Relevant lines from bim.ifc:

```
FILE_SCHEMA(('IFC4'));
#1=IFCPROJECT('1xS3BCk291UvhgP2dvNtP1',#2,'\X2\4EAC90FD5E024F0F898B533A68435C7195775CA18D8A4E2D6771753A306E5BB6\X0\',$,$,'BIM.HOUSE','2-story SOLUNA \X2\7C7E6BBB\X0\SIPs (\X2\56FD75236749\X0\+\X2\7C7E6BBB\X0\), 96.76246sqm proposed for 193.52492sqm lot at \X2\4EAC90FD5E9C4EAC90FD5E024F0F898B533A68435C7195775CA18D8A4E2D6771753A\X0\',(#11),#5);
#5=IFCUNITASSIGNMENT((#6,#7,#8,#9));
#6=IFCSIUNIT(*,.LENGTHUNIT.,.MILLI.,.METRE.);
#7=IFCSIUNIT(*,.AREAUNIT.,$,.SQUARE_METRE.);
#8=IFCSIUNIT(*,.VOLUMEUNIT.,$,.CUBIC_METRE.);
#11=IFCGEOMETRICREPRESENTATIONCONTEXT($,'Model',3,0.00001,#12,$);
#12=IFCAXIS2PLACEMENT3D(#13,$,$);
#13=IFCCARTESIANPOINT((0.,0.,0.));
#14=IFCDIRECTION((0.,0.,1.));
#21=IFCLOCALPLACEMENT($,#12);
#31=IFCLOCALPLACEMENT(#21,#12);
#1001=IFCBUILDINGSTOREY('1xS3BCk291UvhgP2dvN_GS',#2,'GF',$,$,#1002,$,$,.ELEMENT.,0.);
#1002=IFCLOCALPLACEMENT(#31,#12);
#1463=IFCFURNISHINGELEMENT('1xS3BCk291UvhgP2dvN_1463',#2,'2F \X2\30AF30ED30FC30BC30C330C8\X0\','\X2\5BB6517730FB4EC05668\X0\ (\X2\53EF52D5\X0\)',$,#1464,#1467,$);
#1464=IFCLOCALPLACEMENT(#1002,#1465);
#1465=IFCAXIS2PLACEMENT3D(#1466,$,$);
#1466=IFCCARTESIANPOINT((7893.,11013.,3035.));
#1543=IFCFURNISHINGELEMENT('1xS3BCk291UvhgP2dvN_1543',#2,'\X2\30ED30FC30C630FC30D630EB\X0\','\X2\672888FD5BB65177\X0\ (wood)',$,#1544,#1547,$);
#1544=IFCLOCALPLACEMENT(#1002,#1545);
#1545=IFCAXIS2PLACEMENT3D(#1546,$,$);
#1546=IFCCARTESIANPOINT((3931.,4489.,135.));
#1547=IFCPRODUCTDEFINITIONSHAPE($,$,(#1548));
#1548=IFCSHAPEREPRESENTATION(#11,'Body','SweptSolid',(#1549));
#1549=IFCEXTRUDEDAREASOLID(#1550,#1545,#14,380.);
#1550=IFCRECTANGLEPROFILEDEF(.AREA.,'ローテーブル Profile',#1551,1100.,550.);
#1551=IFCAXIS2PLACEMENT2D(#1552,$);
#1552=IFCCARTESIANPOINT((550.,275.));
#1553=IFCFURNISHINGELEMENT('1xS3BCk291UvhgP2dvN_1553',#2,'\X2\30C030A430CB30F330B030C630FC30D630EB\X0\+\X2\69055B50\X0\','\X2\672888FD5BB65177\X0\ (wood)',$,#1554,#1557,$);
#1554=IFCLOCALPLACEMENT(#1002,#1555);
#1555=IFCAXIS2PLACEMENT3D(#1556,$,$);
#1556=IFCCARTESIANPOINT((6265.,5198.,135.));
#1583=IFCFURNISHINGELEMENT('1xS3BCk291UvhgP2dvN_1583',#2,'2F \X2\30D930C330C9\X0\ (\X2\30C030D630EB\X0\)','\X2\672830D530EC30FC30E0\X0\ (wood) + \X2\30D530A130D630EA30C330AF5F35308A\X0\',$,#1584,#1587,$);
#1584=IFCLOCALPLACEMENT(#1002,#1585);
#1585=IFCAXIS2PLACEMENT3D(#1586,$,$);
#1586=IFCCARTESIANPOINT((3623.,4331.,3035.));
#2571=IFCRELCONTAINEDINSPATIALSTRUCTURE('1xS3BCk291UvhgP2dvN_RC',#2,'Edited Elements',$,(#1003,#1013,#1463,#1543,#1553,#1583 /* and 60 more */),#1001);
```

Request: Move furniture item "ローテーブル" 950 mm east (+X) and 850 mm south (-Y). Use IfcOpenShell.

```python
import ifcopenshell
import ifcopenshell.api.geometry
import ifcopenshell.util.placement

model = ifcopenshell.open("bim.ifc")

item = model.by_guid("1xS3BCk291UvhgP2dvN_1543")
matrix = ifcopenshell.util.placement.get_local_placement(item.ObjectPlacement)
matrix[0, 3] += 950.0
matrix[1, 3] -= 850.0
ifcopenshell.api.geometry.edit_object_placement(model, product=item, matrix=matrix, is_si=False)

print(ifcopenshell.util.placement.get_local_placement(item.ObjectPlacement).round(3) + 0.0)

model.write("bim-out.ifc")
```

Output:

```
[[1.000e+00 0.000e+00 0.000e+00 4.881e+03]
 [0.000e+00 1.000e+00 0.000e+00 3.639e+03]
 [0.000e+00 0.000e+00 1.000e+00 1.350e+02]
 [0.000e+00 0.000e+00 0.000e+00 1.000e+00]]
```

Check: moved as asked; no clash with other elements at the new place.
